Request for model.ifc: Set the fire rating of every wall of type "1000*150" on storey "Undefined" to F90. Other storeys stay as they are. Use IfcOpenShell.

First a look at what the model holds.

```python
import ifcopenshell
import ifcopenshell.util.element

model = ifcopenshell.open("model.ifc")
print(model.schema)
storey = next(s for s in model.by_type("IfcBuildingStorey") if s.Name == "Undefined")
walls = [e for e in ifcopenshell.util.element.get_decomposition(storey) if e.is_a("IfcWall")]
seen = {}
for e in walls:
    element_type = ifcopenshell.util.element.get_type(e)
    key = (element_type.Name if element_type != e and element_type else None, ifcopenshell.util.element.get_pset(e, "Pset_WallCommon", "FireRating"))
    seen[key] = seen.get(key, 0) + 1
for (name, value), count in sorted(seen.items(), key=str):
    print(count, "x", name, "|", value)
```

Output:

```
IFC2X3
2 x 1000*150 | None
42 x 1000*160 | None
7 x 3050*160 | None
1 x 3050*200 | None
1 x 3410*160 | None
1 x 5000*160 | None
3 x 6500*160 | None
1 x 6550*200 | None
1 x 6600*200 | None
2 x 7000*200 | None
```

```python
import ifcopenshell
import ifcopenshell.api.pset
import ifcopenshell.util.element

model = ifcopenshell.open("model.ifc")

storey = next(s for s in model.by_type("IfcBuildingStorey") if s.Name == "Undefined")
walls = [e for e in ifcopenshell.util.element.get_decomposition(storey) if e.is_a("IfcWall")]

count = 0
for e in walls:
    element_type = ifcopenshell.util.element.get_type(e)
    if element_type in (None, e) or element_type.Name != "1000*150":
        continue
    # add_pset returns the element's existing set when there is one.
    pset = ifcopenshell.api.pset.add_pset(model, product=e, name="Pset_WallCommon")
    ifcopenshell.api.pset.edit_pset(model, pset=pset, properties={"FireRating": "F90"})
    count += 1

print(count, "walls updated")

model.write("model_rev.ifc")
```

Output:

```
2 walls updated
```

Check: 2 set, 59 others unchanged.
